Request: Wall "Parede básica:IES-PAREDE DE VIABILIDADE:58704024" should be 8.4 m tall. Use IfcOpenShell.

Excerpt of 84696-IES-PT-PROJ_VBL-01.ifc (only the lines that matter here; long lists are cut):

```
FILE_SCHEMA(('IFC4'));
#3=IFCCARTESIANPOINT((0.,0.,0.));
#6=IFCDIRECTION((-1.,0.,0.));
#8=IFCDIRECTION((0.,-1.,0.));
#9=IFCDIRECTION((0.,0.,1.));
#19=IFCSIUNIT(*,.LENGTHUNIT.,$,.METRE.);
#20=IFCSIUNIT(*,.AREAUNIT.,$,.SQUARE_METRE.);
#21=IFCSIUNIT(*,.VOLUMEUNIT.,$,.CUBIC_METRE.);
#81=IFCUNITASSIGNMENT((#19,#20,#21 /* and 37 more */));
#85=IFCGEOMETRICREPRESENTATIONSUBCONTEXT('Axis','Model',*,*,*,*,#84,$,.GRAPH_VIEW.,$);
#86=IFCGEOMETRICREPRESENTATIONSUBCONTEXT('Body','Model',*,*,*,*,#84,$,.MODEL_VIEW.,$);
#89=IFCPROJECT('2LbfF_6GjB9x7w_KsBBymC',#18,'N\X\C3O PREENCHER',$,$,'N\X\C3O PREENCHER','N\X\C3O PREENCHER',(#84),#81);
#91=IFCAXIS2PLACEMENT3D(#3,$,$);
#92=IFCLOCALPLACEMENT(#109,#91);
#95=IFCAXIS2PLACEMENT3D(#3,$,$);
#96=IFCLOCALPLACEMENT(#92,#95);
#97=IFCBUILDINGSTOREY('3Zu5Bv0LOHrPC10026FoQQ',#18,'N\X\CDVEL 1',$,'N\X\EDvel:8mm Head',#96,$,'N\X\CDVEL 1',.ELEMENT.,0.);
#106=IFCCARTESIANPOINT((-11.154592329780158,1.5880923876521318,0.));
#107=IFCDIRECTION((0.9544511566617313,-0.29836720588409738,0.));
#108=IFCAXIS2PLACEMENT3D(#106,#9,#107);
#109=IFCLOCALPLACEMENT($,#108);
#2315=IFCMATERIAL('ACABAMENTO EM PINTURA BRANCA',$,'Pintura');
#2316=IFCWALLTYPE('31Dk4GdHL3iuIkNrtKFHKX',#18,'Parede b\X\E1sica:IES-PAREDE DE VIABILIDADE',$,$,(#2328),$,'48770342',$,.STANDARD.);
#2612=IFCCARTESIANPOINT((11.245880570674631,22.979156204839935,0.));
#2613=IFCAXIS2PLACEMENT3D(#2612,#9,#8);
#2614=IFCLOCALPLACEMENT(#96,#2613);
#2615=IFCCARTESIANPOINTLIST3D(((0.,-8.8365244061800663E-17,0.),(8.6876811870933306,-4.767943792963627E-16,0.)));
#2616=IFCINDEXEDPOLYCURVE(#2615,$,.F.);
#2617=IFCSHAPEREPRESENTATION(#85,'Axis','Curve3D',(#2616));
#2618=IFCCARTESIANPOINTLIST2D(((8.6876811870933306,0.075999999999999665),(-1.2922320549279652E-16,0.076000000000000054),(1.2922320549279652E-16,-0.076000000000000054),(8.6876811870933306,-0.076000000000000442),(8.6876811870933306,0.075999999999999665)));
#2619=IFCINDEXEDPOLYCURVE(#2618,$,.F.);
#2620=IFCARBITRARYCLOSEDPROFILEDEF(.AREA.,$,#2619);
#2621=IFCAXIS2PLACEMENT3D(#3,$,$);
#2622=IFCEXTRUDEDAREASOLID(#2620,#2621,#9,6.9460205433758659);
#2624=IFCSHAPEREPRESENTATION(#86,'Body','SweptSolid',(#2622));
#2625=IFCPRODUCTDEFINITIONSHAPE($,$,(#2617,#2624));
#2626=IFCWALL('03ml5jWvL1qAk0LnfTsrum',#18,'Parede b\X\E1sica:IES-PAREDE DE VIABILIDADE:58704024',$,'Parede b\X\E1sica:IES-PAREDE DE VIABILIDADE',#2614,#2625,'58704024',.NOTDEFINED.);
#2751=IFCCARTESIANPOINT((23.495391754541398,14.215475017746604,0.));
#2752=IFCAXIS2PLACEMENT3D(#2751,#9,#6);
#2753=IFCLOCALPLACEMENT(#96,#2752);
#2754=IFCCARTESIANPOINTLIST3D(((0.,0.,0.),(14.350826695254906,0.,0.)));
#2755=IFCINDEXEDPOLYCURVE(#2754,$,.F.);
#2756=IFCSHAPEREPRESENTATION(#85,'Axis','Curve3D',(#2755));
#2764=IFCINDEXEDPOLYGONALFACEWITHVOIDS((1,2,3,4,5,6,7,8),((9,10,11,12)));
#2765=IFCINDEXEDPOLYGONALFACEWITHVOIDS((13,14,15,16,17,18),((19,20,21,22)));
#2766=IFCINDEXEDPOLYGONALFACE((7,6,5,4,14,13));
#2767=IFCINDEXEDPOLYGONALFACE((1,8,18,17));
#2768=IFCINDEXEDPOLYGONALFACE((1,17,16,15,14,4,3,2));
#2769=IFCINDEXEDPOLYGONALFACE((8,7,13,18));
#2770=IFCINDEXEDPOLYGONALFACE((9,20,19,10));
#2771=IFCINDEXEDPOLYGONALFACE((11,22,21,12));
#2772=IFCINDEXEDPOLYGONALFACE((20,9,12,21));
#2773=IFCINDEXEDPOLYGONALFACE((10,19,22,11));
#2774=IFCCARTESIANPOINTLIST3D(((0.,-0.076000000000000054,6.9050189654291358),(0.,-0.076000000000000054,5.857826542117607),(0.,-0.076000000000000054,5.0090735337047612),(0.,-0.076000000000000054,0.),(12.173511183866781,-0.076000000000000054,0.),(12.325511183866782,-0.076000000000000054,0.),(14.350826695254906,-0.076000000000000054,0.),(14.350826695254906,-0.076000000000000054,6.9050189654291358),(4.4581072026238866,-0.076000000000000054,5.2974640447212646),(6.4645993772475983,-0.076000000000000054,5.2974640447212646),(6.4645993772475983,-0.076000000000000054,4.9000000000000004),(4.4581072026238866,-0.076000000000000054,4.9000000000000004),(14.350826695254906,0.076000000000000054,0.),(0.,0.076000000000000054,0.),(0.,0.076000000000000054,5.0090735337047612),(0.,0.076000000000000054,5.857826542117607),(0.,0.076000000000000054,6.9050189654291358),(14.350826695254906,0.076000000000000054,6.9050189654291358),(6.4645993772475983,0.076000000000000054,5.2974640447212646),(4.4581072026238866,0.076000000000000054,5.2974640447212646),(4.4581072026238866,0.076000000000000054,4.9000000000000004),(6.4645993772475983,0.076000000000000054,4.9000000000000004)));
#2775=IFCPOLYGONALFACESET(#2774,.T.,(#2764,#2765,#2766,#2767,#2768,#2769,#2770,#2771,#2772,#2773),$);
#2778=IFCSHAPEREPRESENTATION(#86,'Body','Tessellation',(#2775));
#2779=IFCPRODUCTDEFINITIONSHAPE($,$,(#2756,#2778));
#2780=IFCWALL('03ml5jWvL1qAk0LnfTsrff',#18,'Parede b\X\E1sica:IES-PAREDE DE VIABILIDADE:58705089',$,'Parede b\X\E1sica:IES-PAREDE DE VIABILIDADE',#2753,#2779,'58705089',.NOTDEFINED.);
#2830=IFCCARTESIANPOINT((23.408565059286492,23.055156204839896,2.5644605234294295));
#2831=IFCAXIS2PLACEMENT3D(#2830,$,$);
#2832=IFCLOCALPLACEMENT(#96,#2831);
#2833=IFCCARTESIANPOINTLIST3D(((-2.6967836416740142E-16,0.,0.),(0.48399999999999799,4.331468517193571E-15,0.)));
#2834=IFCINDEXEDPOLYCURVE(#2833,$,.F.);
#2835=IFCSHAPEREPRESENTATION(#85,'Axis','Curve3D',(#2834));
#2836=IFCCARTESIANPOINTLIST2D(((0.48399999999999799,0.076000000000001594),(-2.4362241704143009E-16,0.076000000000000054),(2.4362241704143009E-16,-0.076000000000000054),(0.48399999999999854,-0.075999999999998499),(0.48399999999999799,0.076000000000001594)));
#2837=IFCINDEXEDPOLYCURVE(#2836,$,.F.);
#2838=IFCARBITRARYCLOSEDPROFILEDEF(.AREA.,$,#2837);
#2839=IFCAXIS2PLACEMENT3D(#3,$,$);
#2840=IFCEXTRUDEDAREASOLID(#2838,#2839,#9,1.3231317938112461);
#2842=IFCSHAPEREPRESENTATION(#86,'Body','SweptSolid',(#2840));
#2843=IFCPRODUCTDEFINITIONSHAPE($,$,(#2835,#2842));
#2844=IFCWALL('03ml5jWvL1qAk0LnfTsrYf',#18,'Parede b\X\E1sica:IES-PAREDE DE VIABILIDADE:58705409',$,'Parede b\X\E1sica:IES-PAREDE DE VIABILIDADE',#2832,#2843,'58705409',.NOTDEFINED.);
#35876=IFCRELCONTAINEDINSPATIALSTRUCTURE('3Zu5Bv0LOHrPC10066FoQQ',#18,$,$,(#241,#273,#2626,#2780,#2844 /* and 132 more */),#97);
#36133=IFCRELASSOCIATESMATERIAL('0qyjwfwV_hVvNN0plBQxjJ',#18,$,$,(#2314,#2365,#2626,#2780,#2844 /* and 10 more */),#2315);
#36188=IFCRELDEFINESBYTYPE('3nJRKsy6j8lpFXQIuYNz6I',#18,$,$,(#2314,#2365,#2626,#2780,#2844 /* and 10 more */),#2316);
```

```python
import ifcopenshell
import ifcopenshell.geom
import ifcopenshell.util.representation
import ifcopenshell.util.shape

model = ifcopenshell.open("84696-IES-PT-PROJ_VBL-01.ifc")
settings = ifcopenshell.geom.settings()


def volume(element):
    """Net volume in cubic metres, openings subtracted."""
    shape = ifcopenshell.geom.create_shape(settings, element)
    return ifcopenshell.util.shape.get_volume(shape.geometry)


wall = model.by_guid("03ml5jWvL1qAk0LnfTsrum")
before = volume(wall)

body = ifcopenshell.util.representation.get_representation(wall, "Model", "Body")
solid = body.Items[0]
old_height = solid.Depth
solid.Depth = 8.4
after = volume(wall)

print(f"height {old_height:g} -> {solid.Depth:g}, volume {before:.3f} -> {after:.3f} m3")

model.write("84696-IES-PT-PROJ_VBL-01_edited.ifc")
```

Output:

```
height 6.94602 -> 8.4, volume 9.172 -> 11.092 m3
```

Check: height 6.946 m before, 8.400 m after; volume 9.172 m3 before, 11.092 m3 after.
